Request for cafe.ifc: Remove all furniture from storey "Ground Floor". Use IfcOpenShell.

First a look at what the model holds.

```python
import ifcopenshell
import ifcopenshell.util.element

model = ifcopenshell.open("cafe.ifc")
print(model.schema)
storey = next(s for s in model.by_type("IfcBuildingStorey") if s.Name == "Ground Floor")
furniture = [e for e in ifcopenshell.util.element.get_decomposition(storey) if e.is_a("IfcFurnishingElement")]
seen = {}
for e in furniture:
    element_type = ifcopenshell.util.element.get_type(e)
    name = element_type.Name if element_type not in (None, e) else None
    seen[name] = seen.get(name, 0) + 1
for name, count in sorted(seen.items(), key=str):
    print(count, "x", name)
```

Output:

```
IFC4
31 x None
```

```python
import ifcopenshell
import ifcopenshell.api.root
import ifcopenshell.util.element

model = ifcopenshell.open("cafe.ifc")

storey = next(s for s in model.by_type("IfcBuildingStorey") if s.Name == "Ground Floor")
furniture = [e for e in ifcopenshell.util.element.get_decomposition(storey) if e.is_a("IfcFurnishingElement")]

for e in furniture:
    ifcopenshell.api.root.remove_product(model, product=e)
print(len(furniture), "removed")

model.write("cafe_edited.ifc")
```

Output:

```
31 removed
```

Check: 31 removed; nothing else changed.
